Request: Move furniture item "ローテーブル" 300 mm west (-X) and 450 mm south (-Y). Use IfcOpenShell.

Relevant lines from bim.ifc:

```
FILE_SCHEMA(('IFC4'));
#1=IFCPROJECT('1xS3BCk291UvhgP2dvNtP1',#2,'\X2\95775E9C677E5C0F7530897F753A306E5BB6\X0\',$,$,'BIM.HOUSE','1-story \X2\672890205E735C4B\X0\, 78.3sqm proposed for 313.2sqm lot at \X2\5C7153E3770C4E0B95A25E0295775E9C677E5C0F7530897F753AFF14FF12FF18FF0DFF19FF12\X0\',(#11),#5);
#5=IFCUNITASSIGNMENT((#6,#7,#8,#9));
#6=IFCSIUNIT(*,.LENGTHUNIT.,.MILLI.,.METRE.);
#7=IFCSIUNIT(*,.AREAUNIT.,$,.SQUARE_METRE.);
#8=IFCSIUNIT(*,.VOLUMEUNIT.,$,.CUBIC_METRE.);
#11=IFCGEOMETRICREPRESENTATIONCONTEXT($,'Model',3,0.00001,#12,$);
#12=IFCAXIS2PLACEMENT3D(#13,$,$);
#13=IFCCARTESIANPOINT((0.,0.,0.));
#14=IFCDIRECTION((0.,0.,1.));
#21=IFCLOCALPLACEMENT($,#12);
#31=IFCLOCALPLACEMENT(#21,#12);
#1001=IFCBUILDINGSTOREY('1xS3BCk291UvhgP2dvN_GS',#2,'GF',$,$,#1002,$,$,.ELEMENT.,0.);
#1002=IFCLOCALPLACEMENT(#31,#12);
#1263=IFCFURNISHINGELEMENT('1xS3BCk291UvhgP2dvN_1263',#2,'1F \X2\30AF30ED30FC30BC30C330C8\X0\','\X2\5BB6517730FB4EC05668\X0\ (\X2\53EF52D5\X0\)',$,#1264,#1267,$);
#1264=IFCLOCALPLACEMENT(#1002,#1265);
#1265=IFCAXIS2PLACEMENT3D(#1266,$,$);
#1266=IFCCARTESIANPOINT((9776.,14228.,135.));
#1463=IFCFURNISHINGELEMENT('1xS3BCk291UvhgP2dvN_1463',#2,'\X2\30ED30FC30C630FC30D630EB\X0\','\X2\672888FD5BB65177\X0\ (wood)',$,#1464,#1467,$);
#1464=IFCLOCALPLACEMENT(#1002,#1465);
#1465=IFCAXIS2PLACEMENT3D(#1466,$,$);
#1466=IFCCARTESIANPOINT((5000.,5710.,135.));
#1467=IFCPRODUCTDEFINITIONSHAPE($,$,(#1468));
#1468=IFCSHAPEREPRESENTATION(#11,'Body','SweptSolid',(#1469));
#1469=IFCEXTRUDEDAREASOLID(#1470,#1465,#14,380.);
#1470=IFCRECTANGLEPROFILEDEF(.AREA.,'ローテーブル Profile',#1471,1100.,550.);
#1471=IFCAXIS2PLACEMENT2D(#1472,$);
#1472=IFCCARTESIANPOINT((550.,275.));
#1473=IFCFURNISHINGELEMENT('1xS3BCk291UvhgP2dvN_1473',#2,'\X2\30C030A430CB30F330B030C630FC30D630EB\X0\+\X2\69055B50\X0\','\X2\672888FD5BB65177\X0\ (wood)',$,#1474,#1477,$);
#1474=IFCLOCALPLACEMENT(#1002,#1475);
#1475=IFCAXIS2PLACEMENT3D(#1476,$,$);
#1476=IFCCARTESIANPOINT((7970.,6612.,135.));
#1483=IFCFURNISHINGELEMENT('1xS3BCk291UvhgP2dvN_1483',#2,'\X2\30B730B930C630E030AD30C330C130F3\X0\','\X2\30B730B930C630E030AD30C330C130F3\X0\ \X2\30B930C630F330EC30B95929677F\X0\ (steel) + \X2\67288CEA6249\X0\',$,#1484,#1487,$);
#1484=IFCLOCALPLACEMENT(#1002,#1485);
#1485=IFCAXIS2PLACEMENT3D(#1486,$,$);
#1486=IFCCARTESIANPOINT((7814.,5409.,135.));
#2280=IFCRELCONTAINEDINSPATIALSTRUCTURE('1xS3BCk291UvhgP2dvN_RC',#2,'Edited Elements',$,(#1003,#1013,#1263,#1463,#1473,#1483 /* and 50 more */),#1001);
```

```python
import ifcopenshell
import ifcopenshell.api.geometry
import ifcopenshell.util.placement

model = ifcopenshell.open("bim.ifc")

item = model.by_guid("1xS3BCk291UvhgP2dvN_1463")
matrix = ifcopenshell.util.placement.get_local_placement(item.ObjectPlacement)
matrix[0, 3] -= 300.0
matrix[1, 3] -= 450.0
ifcopenshell.api.geometry.edit_object_placement(model, product=item, matrix=matrix, is_si=False)

print(ifcopenshell.util.placement.get_local_placement(item.ObjectPlacement).round(3) + 0.0)

model.write("bim_rev.ifc")
```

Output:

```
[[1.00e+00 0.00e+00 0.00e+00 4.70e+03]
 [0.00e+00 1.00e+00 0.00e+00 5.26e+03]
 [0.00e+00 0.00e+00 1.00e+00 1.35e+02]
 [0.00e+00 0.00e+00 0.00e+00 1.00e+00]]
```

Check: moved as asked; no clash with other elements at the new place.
